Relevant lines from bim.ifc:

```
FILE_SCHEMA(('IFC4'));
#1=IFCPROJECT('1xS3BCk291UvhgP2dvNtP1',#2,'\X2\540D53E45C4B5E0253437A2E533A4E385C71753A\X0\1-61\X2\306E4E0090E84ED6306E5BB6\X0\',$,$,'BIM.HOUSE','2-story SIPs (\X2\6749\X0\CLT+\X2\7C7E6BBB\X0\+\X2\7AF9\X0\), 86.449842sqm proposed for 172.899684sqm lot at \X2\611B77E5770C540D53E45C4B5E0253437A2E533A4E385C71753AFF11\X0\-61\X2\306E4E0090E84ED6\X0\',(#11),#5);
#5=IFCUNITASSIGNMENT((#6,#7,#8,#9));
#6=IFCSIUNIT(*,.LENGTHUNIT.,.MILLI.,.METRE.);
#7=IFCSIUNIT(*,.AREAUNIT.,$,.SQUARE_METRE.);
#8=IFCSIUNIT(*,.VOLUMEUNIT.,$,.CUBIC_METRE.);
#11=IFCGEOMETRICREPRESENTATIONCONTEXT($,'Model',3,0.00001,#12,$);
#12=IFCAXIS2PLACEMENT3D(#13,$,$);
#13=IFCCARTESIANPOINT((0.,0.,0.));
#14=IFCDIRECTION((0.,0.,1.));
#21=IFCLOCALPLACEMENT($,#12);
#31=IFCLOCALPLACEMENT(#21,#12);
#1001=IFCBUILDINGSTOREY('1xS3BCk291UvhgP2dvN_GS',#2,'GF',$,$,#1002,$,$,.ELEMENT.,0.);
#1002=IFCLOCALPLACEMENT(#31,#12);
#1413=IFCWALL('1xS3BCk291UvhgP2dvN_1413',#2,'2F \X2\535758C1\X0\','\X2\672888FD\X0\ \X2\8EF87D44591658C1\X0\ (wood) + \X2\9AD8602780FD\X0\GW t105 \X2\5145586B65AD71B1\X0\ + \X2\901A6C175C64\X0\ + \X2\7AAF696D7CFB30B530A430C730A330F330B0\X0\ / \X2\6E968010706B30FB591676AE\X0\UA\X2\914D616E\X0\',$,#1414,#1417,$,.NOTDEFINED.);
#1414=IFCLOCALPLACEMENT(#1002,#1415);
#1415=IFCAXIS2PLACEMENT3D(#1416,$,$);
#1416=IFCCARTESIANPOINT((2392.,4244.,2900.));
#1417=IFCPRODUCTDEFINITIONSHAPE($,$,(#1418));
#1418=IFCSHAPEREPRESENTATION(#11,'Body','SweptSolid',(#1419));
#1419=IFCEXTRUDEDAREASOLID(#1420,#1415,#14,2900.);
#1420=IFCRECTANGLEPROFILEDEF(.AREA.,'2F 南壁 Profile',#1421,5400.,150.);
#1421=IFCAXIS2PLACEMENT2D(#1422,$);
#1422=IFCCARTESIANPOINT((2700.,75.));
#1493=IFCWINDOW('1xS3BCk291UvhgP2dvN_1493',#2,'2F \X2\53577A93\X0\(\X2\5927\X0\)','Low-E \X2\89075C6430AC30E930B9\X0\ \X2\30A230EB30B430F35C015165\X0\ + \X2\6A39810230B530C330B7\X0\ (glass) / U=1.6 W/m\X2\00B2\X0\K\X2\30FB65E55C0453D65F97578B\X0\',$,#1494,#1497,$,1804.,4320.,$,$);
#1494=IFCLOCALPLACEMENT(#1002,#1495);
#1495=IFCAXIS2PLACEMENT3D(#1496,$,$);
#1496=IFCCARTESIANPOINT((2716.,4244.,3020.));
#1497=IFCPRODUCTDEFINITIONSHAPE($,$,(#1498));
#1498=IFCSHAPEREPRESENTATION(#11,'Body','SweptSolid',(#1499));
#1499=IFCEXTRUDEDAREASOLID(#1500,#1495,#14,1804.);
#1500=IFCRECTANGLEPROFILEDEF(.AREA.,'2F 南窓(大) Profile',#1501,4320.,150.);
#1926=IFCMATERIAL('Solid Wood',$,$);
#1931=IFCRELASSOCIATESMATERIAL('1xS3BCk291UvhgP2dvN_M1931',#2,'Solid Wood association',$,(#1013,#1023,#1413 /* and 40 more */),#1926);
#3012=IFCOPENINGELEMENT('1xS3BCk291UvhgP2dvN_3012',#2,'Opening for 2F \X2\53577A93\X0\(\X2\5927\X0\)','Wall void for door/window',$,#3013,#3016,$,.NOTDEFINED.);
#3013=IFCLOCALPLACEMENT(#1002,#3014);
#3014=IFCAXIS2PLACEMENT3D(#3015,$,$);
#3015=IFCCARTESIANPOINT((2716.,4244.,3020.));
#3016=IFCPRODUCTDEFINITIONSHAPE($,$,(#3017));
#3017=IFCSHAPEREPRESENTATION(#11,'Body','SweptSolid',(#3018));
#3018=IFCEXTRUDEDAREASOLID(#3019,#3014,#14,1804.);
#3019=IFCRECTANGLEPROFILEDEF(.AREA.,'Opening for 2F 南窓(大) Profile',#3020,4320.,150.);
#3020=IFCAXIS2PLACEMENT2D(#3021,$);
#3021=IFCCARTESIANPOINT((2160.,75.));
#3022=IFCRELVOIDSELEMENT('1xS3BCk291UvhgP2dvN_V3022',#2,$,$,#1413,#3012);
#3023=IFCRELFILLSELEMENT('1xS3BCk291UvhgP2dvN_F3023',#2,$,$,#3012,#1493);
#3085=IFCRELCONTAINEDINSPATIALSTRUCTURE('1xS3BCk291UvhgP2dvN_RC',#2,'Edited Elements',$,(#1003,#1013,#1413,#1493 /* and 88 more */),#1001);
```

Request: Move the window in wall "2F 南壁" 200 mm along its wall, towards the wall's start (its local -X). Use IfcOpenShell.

```python
import ifcopenshell
import ifcopenshell.api.geometry
import ifcopenshell.util.placement
import ifcopenshell.util.unit

model = ifcopenshell.open("bim.ifc")
unit_scale = ifcopenshell.util.unit.calculate_unit_scale(model)

window = model.by_guid("1xS3BCk291UvhgP2dvN_1493")
opening = window.FillsVoids[0].RelatingOpeningElement
wall = opening.VoidsElements[0].RelatingBuildingElement

wall_matrix = ifcopenshell.util.placement.get_local_placement(wall.ObjectPlacement)
shift = wall_matrix[:3, 0] * -0.2 / unit_scale
before = ifcopenshell.util.placement.get_local_placement(window.ObjectPlacement)[:3, 3].copy()

# The window is not placed relative to its opening, so move both.
for product in (opening, window):
    matrix = ifcopenshell.util.placement.get_local_placement(product.ObjectPlacement)
    matrix[:3, 3] += shift
    ifcopenshell.api.geometry.edit_object_placement(model, product=product, matrix=matrix, is_si=False)

after = ifcopenshell.util.placement.get_local_placement(window.ObjectPlacement)[:3, 3]
print("window moved by", (after - before).round(3) + 0.0)

model.write("bim_edited.ifc")
```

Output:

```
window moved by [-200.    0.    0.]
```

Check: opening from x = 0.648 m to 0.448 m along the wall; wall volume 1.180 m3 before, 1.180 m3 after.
